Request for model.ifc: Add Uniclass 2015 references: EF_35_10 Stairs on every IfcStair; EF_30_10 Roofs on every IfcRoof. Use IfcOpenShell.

First a look at what the model holds.

```python
import ifcopenshell

model = ifcopenshell.open("model.ifc")
print(model.schema)
print("classifications:", [c.Name for c in model.by_type("IfcClassification")])
for ifc_class in ("IfcDoor", "IfcRoof", "IfcStair", "IfcWall", "IfcWindow"):
    print(ifc_class, len(model.by_type(ifc_class)))
```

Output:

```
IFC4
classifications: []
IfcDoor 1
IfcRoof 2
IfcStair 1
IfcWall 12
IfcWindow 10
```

```python
import ifcopenshell
import ifcopenshell.api.classification

model = ifcopenshell.open("model.ifc")

system = ifcopenshell.api.classification.add_classification(model, classification="Uniclass 2015")

codes = {
    "IfcStair": ("EF_35_10", "Stairs"),
    "IfcRoof": ("EF_30_10", "Roofs"),
}
for ifc_class, (code, name) in codes.items():
    products = model.by_type(ifc_class)
    ifcopenshell.api.classification.add_reference(
        model, products=products, classification=system, identification=code, name=name
    )
    print(code, len(products))

model.write("model_rev.ifc")
```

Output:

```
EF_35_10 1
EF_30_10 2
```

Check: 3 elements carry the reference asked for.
